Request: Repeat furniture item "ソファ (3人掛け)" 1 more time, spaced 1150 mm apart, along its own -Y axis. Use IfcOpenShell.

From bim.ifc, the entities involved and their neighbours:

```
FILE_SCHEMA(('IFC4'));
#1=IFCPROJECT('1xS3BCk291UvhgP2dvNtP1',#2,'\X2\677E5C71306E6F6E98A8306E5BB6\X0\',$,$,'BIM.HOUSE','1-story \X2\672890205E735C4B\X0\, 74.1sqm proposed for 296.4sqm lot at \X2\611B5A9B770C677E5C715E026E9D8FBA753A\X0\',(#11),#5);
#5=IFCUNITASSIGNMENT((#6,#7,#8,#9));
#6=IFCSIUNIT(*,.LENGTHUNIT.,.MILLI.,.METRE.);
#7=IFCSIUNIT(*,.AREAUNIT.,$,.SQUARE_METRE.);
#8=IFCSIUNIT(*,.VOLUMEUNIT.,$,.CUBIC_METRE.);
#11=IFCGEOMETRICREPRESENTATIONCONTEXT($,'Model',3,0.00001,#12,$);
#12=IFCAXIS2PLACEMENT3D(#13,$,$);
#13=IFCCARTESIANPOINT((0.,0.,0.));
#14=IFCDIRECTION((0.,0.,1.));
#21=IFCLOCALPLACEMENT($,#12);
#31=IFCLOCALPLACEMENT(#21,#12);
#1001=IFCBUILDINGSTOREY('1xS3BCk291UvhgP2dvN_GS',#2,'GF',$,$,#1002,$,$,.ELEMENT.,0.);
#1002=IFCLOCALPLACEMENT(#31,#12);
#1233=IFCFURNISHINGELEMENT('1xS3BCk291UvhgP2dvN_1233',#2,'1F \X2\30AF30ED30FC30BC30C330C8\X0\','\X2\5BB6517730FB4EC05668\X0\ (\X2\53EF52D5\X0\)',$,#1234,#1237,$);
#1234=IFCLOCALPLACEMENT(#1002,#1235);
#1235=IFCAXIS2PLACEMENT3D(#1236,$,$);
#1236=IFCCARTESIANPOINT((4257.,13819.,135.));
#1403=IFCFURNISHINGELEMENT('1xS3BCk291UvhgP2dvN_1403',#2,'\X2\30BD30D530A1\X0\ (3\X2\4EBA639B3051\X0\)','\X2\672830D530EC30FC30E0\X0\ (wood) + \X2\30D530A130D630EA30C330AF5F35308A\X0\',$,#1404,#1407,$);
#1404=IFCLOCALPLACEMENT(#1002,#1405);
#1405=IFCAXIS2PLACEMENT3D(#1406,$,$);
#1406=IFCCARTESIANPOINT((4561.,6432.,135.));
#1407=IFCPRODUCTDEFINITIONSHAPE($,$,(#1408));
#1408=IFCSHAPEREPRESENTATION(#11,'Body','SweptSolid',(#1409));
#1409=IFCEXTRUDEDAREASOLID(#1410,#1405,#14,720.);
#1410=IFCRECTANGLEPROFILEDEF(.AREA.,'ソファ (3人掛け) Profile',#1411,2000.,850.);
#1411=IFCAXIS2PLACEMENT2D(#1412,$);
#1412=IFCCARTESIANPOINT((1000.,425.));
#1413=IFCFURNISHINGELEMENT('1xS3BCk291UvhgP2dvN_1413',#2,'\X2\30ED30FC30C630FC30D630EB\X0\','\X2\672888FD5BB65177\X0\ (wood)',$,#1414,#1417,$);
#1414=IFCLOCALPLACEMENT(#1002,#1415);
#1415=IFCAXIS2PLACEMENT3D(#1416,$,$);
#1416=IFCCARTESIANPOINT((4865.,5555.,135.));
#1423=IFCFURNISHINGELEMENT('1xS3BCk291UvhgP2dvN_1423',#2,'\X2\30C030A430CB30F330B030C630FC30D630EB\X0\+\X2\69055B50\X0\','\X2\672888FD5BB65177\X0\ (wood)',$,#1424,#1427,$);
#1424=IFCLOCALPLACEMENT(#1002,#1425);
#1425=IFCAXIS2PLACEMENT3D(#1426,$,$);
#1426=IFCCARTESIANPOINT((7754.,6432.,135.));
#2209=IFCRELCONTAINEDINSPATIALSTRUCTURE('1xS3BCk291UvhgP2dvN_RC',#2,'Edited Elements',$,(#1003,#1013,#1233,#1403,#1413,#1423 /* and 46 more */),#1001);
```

```python
import ifcopenshell
import ifcopenshell.api.geometry
import ifcopenshell.api.root
import ifcopenshell.util.element
import ifcopenshell.util.placement
import ifcopenshell.util.unit

model = ifcopenshell.open("bim.ifc")
unit_scale = ifcopenshell.util.unit.calculate_unit_scale(model)


def reuse_history(source, copy):
    """copy_class also copies each property set's owner history, people and application; keep the originals."""
    for rel in copy.IsDefinedBy:
        if rel.is_a("IfcRelDefinesByProperties") and (history := rel.RelatingPropertyDefinition.OwnerHistory):
            rel.RelatingPropertyDefinition.OwnerHistory = source.OwnerHistory
            ifcopenshell.util.element.remove_deep2(model, history)


source = model.by_guid("1xS3BCk291UvhgP2dvN_1403")
base = ifcopenshell.util.placement.get_local_placement(source.ObjectPlacement)
step = -base[:3, 1] * 1.15 / unit_scale

for i in range(1, 2):
    copy = ifcopenshell.api.root.copy_class(model, product=source)
    copy.Representation = ifcopenshell.util.element.copy_deep(
        model, source.Representation, exclude=["IfcGeometricRepresentationContext", "IfcRepresentationMap"]
    )
    reuse_history(source, copy)
    matrix = base.copy()
    matrix[:3, 3] += i * step
    print("added at", matrix[:3, 3].round(3) + 0.0)
    ifcopenshell.api.geometry.edit_object_placement(model, product=copy, matrix=matrix, is_si=False)

model.write("bim_rev.ifc")
```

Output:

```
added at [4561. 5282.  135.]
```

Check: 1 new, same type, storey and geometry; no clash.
